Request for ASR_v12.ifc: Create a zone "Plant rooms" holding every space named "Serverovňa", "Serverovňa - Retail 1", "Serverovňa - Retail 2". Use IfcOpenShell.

First a look at what the model holds.

```python
import ifcopenshell

model = ifcopenshell.open("ASR_v12.ifc")
print(model.schema)
seen = {}
for space in model.by_type("IfcSpace"):
    seen[space.LongName] = seen.get(space.LongName, 0) + 1
for name, count in sorted(seen.items(), key=str):
    print(count, "x", name)
print("zones:", [z.Name for z in model.by_type("IfcZone")][:20])
```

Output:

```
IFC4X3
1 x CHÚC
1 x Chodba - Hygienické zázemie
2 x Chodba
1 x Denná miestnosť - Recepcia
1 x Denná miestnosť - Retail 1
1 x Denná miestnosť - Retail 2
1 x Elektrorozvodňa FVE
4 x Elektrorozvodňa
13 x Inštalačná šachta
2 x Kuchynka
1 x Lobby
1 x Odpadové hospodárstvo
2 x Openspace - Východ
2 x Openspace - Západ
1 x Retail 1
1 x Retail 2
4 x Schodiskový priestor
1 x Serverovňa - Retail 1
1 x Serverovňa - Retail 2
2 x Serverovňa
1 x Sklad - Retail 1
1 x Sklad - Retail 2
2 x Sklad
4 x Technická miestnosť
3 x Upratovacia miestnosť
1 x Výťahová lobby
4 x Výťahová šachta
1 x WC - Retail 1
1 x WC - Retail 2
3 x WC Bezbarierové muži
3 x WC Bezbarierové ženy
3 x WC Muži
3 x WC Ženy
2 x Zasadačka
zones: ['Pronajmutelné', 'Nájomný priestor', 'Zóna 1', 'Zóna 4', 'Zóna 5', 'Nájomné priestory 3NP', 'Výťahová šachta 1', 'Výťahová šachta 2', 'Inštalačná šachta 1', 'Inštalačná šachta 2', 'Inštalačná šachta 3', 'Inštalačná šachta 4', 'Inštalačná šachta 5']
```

```python
import ifcopenshell
import ifcopenshell.api.group
import ifcopenshell.api.root

model = ifcopenshell.open("ASR_v12.ifc")

names = {"Serverovňa", "Serverovňa - Retail 1", "Serverovňa - Retail 2"}
spaces = [s for s in model.by_type("IfcSpace") if s.LongName in names]

zone = ifcopenshell.api.root.create_entity(model, ifc_class="IfcZone", name="Plant rooms")
ifcopenshell.api.group.assign_group(model, products=spaces, group=zone)
print(len(spaces), "spaces in", zone.Name)

model.write("ASR_v12_rev.ifc")
```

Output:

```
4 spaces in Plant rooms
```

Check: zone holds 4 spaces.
